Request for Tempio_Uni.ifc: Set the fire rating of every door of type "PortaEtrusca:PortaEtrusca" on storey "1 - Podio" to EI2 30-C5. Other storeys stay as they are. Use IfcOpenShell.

First a look at what the model holds.

```python
import ifcopenshell
import ifcopenshell.util.element

model = ifcopenshell.open("Tempio_Uni.ifc")
print(model.schema)
storey = next(s for s in model.by_type("IfcBuildingStorey") if s.Name == "1 - Podio")
doors = [e for e in ifcopenshell.util.element.get_decomposition(storey) if e.is_a("IfcDoor")]
seen = {}
for e in doors:
    element_type = ifcopenshell.util.element.get_type(e)
    key = (element_type.Name if element_type != e and element_type else None, ifcopenshell.util.element.get_pset(e, "Pset_DoorCommon", "FireRating"))
    seen[key] = seen.get(key, 0) + 1
for (name, value), count in sorted(seen.items(), key=str):
    print(count, "x", name, "|", value)
```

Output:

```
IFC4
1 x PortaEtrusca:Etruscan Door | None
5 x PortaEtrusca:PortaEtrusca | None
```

```python
import ifcopenshell
import ifcopenshell.api.pset
import ifcopenshell.util.element

model = ifcopenshell.open("Tempio_Uni.ifc")

storey = next(s for s in model.by_type("IfcBuildingStorey") if s.Name == "1 - Podio")
doors = [e for e in ifcopenshell.util.element.get_decomposition(storey) if e.is_a("IfcDoor")]

count = 0
for e in doors:
    element_type = ifcopenshell.util.element.get_type(e)
    if element_type in (None, e) or element_type.Name != "PortaEtrusca:PortaEtrusca":
        continue
    # add_pset returns the element's existing set when there is one.
    pset = ifcopenshell.api.pset.add_pset(model, product=e, name="Pset_DoorCommon")
    ifcopenshell.api.pset.edit_pset(model, pset=pset, properties={"FireRating": "EI2 30-C5"})
    count += 1

print(count, "doors updated")

model.write("Tempio_Uni_v2.ifc")
```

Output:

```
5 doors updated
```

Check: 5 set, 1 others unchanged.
